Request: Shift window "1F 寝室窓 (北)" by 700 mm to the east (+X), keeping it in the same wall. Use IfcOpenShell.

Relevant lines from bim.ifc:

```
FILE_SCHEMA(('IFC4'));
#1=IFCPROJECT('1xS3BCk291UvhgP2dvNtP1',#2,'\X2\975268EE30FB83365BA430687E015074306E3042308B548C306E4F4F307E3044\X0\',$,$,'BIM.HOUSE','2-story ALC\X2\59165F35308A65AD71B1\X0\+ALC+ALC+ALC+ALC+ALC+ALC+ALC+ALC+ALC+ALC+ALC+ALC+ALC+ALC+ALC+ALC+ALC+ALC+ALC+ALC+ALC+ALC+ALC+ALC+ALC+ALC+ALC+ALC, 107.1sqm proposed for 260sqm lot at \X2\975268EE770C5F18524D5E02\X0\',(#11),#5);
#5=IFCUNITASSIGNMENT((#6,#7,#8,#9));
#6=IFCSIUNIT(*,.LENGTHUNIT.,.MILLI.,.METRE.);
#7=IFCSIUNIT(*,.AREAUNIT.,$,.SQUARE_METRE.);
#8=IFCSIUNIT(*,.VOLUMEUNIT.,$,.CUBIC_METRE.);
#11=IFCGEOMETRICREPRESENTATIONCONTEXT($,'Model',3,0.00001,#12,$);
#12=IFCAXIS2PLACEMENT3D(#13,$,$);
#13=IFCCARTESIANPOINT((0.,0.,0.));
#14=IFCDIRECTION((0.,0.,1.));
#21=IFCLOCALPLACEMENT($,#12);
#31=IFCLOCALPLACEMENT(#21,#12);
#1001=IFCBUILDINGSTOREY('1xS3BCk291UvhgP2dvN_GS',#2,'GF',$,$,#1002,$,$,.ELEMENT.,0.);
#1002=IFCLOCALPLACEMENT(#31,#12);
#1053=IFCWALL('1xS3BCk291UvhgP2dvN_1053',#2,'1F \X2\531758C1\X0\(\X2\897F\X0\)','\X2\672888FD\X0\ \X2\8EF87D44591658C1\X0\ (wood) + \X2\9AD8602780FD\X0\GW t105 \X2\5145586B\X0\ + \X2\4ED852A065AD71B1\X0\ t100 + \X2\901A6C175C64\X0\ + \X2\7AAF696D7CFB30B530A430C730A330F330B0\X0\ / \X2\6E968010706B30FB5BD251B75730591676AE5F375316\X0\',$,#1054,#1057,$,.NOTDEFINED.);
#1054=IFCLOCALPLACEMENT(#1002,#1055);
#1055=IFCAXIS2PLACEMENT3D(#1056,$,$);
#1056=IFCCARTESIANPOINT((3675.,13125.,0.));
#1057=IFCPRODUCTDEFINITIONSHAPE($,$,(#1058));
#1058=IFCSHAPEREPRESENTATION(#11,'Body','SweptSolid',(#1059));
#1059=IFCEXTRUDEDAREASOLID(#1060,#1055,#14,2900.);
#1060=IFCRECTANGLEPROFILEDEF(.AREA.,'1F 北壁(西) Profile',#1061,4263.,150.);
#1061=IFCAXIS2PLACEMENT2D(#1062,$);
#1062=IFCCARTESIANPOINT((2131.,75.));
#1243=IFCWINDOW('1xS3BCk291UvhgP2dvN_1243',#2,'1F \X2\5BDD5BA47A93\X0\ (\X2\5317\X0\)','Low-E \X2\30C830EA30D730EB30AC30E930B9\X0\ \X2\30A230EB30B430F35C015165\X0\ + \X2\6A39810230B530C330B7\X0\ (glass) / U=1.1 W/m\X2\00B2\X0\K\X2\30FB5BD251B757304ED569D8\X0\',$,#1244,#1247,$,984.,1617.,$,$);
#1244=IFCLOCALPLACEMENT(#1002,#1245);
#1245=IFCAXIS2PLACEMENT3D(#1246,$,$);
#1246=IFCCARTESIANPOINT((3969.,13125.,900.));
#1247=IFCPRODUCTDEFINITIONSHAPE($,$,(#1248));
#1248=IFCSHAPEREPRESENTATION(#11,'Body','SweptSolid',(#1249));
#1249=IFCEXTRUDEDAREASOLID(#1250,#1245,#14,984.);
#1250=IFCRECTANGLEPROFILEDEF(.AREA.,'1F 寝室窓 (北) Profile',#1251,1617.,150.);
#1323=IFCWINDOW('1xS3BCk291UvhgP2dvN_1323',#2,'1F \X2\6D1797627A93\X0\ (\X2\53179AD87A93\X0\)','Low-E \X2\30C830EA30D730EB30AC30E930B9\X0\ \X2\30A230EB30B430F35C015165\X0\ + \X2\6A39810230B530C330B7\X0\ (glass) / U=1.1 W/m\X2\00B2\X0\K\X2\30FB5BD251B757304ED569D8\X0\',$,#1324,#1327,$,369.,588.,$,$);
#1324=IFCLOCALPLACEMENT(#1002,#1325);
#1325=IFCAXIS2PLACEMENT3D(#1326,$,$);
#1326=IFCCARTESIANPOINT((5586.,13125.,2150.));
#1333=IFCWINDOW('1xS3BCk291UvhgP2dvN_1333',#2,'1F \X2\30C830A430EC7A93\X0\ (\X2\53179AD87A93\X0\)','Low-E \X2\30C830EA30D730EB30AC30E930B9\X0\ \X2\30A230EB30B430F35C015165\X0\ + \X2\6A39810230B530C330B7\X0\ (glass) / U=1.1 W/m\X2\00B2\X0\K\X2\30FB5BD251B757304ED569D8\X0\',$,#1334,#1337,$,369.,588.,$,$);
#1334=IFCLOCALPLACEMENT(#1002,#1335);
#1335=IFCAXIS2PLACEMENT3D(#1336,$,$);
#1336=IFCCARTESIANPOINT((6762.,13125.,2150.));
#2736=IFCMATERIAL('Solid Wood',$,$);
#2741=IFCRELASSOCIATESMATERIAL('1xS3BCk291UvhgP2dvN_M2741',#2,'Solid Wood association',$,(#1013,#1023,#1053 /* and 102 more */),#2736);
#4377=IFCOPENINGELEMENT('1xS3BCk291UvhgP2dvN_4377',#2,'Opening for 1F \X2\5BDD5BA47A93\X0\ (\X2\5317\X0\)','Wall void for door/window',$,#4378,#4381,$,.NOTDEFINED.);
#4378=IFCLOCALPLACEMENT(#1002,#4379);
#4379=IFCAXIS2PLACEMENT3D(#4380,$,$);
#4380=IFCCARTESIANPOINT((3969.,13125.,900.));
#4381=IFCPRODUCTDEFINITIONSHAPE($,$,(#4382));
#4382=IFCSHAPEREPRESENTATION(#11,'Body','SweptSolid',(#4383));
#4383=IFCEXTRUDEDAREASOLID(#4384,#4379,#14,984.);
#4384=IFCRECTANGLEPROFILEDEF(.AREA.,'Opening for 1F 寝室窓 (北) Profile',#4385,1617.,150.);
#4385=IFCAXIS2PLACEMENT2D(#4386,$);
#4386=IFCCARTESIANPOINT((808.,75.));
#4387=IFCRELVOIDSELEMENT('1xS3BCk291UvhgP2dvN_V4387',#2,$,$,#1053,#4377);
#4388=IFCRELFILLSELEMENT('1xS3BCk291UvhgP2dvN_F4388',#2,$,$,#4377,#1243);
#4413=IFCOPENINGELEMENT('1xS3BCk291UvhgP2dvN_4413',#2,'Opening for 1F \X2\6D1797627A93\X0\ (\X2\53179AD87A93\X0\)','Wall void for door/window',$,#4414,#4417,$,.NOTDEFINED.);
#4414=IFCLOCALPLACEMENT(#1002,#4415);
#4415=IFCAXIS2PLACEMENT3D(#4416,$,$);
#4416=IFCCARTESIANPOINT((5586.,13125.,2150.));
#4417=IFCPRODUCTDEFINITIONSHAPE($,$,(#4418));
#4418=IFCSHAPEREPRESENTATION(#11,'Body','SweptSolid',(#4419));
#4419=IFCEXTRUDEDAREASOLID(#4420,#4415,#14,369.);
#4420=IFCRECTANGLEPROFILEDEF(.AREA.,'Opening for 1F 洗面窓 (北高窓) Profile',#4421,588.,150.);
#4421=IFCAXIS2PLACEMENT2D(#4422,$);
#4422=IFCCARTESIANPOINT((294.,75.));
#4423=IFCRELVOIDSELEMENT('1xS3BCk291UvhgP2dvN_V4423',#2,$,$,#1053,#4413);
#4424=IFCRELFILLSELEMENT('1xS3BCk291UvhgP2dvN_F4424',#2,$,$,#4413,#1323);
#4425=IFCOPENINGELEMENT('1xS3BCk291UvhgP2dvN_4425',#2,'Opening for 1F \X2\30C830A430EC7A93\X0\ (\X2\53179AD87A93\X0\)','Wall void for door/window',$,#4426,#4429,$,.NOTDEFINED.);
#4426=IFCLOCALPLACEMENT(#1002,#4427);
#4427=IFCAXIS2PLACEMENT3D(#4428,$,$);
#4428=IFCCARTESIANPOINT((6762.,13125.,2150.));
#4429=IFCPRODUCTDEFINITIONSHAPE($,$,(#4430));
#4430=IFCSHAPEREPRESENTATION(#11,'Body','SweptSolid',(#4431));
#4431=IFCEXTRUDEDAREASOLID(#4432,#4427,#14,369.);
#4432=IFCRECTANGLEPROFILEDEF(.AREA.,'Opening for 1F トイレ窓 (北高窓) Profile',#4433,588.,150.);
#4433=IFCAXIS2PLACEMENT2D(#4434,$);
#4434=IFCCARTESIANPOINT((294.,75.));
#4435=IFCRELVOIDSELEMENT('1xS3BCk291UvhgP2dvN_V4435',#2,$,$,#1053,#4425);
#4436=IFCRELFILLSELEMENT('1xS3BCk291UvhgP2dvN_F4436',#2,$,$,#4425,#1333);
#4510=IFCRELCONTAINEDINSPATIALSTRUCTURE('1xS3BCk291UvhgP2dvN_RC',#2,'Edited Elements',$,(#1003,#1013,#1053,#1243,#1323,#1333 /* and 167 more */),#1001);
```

```python
import ifcopenshell
import ifcopenshell.api.geometry
import ifcopenshell.util.placement

model = ifcopenshell.open("bim.ifc")

window = model.by_id(1243)
opening = window.FillsVoids[0].RelatingOpeningElement
wall = opening.VoidsElements[0].RelatingBuildingElement

wall_matrix = ifcopenshell.util.placement.get_local_placement(wall.ObjectPlacement)
shift = wall_matrix[:3, 0] * 700.0
before = ifcopenshell.util.placement.get_local_placement(window.ObjectPlacement)[:3, 3].copy()

# The window is not placed relative to its opening, so move both.
for product in (opening, window):
    matrix = ifcopenshell.util.placement.get_local_placement(product.ObjectPlacement)
    matrix[:3, 3] += shift
    ifcopenshell.api.geometry.edit_object_placement(model, product=product, matrix=matrix, is_si=False)

after = ifcopenshell.util.placement.get_local_placement(window.ObjectPlacement)[:3, 3]
print("window moved by", (after - before).round(3) + 0.0)

model.write("bim_rev.ifc")
```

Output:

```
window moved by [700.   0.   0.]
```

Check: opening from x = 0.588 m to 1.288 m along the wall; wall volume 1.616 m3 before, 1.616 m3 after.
